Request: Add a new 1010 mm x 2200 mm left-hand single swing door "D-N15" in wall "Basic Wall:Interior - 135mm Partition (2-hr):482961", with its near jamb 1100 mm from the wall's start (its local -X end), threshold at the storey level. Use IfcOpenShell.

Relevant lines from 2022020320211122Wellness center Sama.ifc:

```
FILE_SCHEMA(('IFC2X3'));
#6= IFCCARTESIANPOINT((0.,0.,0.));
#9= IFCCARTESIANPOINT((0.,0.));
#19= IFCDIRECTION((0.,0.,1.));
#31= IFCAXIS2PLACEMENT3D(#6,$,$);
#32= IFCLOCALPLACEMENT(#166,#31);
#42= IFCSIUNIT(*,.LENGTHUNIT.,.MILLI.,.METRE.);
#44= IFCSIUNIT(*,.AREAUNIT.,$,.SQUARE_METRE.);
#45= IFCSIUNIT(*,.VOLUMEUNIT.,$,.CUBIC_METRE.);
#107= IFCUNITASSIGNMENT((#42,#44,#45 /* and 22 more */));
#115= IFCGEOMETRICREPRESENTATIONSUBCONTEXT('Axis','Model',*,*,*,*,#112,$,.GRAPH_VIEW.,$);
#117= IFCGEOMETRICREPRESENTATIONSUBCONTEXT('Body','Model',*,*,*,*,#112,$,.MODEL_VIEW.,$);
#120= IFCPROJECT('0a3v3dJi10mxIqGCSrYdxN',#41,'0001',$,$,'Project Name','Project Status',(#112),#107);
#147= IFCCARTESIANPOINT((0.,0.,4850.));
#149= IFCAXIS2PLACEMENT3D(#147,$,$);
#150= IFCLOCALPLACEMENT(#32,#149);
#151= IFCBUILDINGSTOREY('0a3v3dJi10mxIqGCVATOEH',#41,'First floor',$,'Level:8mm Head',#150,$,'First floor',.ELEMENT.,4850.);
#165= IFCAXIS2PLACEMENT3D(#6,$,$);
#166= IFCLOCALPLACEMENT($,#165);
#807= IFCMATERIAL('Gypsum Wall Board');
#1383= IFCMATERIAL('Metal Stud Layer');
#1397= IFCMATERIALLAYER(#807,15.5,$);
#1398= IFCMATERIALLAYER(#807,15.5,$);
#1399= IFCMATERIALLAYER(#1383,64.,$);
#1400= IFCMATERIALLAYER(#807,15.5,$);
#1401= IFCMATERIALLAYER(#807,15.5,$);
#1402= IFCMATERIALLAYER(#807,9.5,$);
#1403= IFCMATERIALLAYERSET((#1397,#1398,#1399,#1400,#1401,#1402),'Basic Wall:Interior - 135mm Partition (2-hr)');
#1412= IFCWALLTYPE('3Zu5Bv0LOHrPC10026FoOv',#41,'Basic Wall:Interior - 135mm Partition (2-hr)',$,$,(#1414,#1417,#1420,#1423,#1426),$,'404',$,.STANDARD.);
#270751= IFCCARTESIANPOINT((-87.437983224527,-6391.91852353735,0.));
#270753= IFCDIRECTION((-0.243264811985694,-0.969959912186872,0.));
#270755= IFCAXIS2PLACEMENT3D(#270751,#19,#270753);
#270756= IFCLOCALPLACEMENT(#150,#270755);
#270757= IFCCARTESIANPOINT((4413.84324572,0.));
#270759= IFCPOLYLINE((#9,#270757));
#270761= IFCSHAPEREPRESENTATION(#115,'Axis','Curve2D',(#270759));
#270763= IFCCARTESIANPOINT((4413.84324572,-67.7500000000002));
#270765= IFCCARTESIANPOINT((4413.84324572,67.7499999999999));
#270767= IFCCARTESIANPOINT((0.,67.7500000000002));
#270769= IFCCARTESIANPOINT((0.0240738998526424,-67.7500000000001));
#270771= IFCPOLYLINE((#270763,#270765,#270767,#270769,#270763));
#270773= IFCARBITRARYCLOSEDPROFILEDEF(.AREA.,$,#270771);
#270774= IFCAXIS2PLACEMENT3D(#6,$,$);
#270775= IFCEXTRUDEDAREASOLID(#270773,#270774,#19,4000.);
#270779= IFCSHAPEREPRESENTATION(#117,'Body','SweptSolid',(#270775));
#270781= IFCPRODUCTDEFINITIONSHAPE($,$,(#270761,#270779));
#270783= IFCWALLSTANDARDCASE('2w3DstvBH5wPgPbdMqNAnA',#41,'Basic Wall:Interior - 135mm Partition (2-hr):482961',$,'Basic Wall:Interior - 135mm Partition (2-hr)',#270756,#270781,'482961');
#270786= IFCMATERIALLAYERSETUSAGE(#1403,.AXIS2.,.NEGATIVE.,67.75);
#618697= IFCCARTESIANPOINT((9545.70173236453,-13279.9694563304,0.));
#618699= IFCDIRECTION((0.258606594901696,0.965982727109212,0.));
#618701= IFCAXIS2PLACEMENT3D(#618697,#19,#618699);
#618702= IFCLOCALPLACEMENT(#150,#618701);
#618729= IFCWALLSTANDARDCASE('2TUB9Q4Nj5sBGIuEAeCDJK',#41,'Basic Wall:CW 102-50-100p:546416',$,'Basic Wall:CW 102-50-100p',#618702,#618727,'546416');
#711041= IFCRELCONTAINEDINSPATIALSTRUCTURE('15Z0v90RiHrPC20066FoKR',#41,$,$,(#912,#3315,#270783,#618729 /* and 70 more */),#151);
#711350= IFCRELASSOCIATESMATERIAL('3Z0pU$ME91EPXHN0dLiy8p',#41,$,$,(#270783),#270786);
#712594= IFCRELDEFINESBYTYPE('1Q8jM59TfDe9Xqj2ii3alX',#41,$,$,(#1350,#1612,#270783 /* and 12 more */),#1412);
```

```python
import numpy as np
import ifcopenshell
import ifcopenshell.api.feature
import ifcopenshell.api.geometry
import ifcopenshell.api.root
import ifcopenshell.api.spatial
import ifcopenshell.api.type
import ifcopenshell.geom
import ifcopenshell.util.element
import ifcopenshell.util.placement
import ifcopenshell.util.representation
import ifcopenshell.util.shape
import ifcopenshell.util.unit

model = ifcopenshell.open("2022020320211122Wellness center Sama.ifc")
unit_scale = ifcopenshell.util.unit.calculate_unit_scale(model)
settings = ifcopenshell.geom.settings()


def volume(element):
    """Net volume in cubic metres, openings subtracted."""
    shape = ifcopenshell.geom.create_shape(settings, element)
    return ifcopenshell.util.shape.get_volume(shape.geometry)


wall = model.by_guid("2w3DstvBH5wPgPbdMqNAnA")
storey = ifcopenshell.util.element.get_container(wall, ifc_class="IfcBuildingStorey")
context = ifcopenshell.util.representation.get_context(model, "Model", "Body", "MODEL_VIEW")
before = volume(wall)

width, height, from_end, sill = 1.01, 2.2, 1.1, 0.0  # metres

# The wall runs along its own X axis, and the end named is its -X end.
wall_shape = ifcopenshell.geom.create_shape(settings, wall)
x, y, z = ifcopenshell.util.shape.get_vertices(wall_shape.geometry).T
start = x.min() + from_end
face, thickness = float(y.min()), float(y.max() - y.min())
wall_matrix = ifcopenshell.util.placement.get_local_placement(wall.ObjectPlacement)
level = ifcopenshell.util.placement.get_local_placement(storey.ObjectPlacement)[2, 3]


def in_wall(x, y):
    """Placement at x, y metres in the wall's axes, at sill height."""
    matrix = wall_matrix.copy()
    matrix[:, 3] = wall_matrix @ np.array([x / unit_scale, y / unit_scale, 0.0, 1.0])
    matrix[2, 3] = level + sill / unit_scale
    return matrix


# Opening: a box that overshoots both wall faces by 50 mm.
opening = ifcopenshell.api.root.create_entity(model, ifc_class="IfcOpeningElement")
box = ifcopenshell.api.geometry.add_wall_representation(
    model, context=context, length=width, height=height, thickness=thickness + 0.1
)
ifcopenshell.api.geometry.assign_representation(model, product=opening, representation=box)
ifcopenshell.api.geometry.edit_object_placement(model, product=opening, matrix=in_wall(start, face - 0.05), is_si=False)
ifcopenshell.api.feature.add_feature(model, feature=opening, element=wall)

door = ifcopenshell.api.root.create_entity(model, ifc_class="IfcDoor", name="D-N15")
door.OverallWidth, door.OverallHeight = width / unit_scale, height / unit_scale
body = ifcopenshell.api.geometry.add_door_representation(
    model,
    context=context,
    overall_width=door.OverallWidth,
    overall_height=door.OverallHeight,
    operation_type="SINGLE_SWING_LEFT",
    lining_properties={"LiningDepth": thickness / unit_scale, "ThresholdDepth": thickness / unit_scale},
)
ifcopenshell.api.geometry.assign_representation(model, product=door, representation=body)
ifcopenshell.api.spatial.assign_container(model, products=[door], relating_structure=storey)
fills = ifcopenshell.api.feature.add_filling(model, opening=opening, element=door)
fills.OwnerHistory = door.OwnerHistory  # required in IFC2X3

# IFC2X3 keeps the operation on the door style.
style = ifcopenshell.api.root.create_entity(model, ifc_class="IfcDoorStyle", name="D-N15")
style.OperationType, style.ConstructionType = "SINGLE_SWING_LEFT", "NOTDEFINED"
style.ParameterTakesPrecedence = style.Sizeable = False
ifcopenshell.api.type.assign_type(model, related_objects=[door], relating_type=style)

# The lining spans the wall, so the door starts at the wall face.
ifcopenshell.api.geometry.edit_object_placement(model, product=door, matrix=in_wall(start, face), is_si=False)

after = volume(wall)

print(f"wall volume {before:.3f} -> {after:.3f} m3")

model.write("2022020320211122Wellness center Sama-out.ifc")
```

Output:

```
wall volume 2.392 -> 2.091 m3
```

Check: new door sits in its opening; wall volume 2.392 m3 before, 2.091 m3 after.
